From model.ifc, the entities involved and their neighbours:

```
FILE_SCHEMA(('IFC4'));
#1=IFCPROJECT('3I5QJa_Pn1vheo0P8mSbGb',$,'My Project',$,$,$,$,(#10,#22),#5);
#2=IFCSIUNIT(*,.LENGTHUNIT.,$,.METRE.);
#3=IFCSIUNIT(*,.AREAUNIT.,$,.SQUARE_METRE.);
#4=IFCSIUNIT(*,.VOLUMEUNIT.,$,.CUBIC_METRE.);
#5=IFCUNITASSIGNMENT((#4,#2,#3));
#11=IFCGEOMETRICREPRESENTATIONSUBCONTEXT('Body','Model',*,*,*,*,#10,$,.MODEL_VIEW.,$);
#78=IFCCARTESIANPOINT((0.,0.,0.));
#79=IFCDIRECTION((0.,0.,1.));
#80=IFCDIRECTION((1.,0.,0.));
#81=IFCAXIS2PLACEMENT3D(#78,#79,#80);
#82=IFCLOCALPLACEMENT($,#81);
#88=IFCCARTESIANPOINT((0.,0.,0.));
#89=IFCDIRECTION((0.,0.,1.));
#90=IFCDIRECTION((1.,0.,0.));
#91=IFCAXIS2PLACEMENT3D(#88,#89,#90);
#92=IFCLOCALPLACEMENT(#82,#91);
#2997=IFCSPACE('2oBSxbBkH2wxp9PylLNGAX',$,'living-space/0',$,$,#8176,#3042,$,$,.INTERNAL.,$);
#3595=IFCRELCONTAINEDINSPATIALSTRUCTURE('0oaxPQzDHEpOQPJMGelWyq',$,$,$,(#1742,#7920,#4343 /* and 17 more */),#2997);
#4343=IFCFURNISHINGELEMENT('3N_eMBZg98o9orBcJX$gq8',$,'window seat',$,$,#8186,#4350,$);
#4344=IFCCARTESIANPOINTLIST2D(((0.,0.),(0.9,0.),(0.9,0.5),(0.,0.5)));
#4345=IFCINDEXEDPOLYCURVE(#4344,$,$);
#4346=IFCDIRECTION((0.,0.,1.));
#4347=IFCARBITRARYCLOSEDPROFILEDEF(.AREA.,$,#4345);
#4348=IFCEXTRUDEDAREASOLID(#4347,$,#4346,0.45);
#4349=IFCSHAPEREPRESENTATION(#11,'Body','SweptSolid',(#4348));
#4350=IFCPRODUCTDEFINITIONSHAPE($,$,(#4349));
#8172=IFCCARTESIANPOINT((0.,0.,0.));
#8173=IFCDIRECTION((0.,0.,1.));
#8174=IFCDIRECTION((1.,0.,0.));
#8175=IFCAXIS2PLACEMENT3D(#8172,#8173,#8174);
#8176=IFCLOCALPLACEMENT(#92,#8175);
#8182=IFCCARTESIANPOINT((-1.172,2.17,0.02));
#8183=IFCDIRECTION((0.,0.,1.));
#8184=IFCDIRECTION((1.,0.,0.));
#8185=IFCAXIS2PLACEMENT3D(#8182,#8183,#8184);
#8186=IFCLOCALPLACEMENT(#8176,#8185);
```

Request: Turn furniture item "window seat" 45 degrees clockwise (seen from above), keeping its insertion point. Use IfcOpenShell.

```python
import ifcopenshell
import ifcopenshell.api.geometry
import ifcopenshell.util.placement

model = ifcopenshell.open("model.ifc")

item = model.by_id(4343)
matrix = ifcopenshell.util.placement.get_local_placement(item.ObjectPlacement)
matrix = matrix @ ifcopenshell.util.placement.rotation(-45, "Z")
ifcopenshell.api.geometry.edit_object_placement(model, product=item, matrix=matrix, is_si=False)

print(ifcopenshell.util.placement.get_local_placement(item.ObjectPlacement).round(3) + 0.0)

model.write("model-out.ifc")
```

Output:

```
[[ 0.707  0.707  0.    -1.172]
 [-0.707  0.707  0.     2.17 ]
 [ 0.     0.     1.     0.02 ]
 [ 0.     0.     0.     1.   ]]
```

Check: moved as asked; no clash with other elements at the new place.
